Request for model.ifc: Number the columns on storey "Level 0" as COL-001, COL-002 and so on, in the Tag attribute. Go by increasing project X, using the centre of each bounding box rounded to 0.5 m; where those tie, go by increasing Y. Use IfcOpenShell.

First a look at what the model holds.

```python
import ifcopenshell
import ifcopenshell.util.element
import ifcopenshell.util.placement

model = ifcopenshell.open("model.ifc")
print(model.schema)
storey = next(s for s in model.by_type("IfcBuildingStorey") if s.Name == "Level 0")
columns = [e for e in ifcopenshell.util.element.get_decomposition(storey) if e.is_a("IfcColumn")]
for e in sorted(columns, key=lambda e: e.id()):
    origin = ifcopenshell.util.placement.get_local_placement(e.ObjectPlacement)[:3, 3]
    print(e.id(), e.Tag, e.Name, origin.round(2) + 0.0, sep=" | ")
```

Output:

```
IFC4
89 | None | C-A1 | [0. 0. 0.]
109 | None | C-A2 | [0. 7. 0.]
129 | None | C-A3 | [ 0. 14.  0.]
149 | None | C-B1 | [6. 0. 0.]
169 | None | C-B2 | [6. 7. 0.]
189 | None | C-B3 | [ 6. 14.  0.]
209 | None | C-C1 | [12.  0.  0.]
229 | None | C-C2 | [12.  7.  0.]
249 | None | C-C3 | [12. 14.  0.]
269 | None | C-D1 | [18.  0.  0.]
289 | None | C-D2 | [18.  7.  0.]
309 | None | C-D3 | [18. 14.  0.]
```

```python
import ifcopenshell
import ifcopenshell.geom
import ifcopenshell.util.element
import ifcopenshell.util.shape

model = ifcopenshell.open("model.ifc")
settings = ifcopenshell.geom.settings()
settings.set("use-world-coords", True)


def centre(element):
    shape = ifcopenshell.geom.create_shape(settings, element)
    return ifcopenshell.util.shape.get_bbox_centroid(shape.geometry)


storey = next(s for s in model.by_type("IfcBuildingStorey") if s.Name == "Level 0")
columns = [e for e in ifcopenshell.util.element.get_decomposition(storey) if e.is_a("IfcColumn")]

# Insertion points can sit at a corner or the storey origin, so sort by the geometry (in metres).
centres = {e: centre(e) for e in columns}
columns.sort(key=lambda e: (round(centres[e][0] / 0.5), centres[e][1]))

for i, e in enumerate(columns, start=1):
    number = f"COL-0{i:02d}"
    e.Tag = number
    print(e.id(), number)

model.write("model_rev.ifc")
```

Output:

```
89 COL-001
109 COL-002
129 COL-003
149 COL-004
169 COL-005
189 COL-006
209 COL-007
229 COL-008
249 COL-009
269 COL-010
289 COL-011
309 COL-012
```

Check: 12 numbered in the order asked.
